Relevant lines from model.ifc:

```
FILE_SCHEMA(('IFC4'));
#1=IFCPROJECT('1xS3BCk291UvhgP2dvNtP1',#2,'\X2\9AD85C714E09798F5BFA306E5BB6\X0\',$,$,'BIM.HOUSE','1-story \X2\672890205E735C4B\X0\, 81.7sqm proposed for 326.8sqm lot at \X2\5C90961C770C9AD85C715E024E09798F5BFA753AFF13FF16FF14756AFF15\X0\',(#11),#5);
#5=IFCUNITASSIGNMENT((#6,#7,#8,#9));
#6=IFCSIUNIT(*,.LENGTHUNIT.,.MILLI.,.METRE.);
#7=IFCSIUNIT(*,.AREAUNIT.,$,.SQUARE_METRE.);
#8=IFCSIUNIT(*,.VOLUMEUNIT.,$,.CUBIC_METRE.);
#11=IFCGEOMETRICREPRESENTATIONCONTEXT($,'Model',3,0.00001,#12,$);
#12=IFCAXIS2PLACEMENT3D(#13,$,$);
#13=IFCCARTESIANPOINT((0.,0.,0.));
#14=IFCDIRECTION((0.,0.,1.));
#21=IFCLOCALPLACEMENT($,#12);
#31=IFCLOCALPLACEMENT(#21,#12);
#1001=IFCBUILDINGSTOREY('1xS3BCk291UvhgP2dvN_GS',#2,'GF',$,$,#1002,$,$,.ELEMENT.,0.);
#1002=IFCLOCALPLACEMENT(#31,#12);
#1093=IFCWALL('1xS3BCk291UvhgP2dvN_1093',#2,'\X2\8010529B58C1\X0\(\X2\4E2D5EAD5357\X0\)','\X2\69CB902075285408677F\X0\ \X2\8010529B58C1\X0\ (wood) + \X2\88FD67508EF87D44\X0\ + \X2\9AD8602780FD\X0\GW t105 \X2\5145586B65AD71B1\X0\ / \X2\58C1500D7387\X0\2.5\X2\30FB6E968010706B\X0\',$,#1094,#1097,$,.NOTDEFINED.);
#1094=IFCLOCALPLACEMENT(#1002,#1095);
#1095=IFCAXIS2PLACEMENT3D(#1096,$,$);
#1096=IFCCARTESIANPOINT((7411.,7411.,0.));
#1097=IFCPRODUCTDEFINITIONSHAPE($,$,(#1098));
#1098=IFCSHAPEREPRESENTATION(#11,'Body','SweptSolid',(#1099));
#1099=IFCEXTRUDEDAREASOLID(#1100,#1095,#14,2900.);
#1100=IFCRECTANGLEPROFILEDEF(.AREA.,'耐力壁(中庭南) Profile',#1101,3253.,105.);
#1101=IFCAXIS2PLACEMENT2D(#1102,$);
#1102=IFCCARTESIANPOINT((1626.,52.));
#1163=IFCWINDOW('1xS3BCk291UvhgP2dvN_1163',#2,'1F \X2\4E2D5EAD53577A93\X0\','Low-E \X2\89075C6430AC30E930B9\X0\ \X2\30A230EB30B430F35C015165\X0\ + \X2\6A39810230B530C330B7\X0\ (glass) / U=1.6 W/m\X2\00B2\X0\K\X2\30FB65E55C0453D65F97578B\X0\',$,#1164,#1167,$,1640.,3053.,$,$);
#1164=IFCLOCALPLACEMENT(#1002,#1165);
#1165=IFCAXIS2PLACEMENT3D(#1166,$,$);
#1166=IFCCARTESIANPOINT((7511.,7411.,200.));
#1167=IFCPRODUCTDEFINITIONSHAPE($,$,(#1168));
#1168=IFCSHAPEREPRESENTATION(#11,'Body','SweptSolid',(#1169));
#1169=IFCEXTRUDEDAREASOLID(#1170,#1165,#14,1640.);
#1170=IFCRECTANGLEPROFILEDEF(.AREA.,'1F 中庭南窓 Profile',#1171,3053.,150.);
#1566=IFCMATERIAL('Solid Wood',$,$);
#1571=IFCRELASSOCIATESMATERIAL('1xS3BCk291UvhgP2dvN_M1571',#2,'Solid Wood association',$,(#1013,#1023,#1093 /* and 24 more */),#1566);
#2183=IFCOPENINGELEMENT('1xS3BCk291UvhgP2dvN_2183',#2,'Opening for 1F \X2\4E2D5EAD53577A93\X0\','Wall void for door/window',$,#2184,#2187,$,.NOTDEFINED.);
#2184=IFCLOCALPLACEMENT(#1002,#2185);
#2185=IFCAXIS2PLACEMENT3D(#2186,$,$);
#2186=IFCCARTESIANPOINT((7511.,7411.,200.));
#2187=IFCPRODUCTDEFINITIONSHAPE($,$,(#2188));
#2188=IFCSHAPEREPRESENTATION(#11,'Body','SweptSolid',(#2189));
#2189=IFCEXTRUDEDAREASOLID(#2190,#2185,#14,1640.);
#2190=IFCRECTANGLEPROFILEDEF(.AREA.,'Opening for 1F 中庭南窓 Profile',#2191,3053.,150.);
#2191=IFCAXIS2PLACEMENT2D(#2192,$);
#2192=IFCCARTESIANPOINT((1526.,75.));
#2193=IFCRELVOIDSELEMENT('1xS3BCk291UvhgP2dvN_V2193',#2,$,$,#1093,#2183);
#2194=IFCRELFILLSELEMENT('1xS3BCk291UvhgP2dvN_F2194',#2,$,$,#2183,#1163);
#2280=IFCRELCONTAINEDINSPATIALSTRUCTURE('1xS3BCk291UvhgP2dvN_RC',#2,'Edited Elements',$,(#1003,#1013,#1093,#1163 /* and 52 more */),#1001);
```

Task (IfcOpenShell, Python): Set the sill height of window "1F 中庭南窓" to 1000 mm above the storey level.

```python
import numpy as np
import ifcopenshell
import ifcopenshell.api.geometry
import ifcopenshell.geom
import ifcopenshell.util.element
import ifcopenshell.util.placement
import ifcopenshell.util.shape
import ifcopenshell.util.unit

model = ifcopenshell.open("model.ifc")
unit_scale = ifcopenshell.util.unit.calculate_unit_scale(model)

window = model.by_guid("1xS3BCk291UvhgP2dvN_1163")
opening = window.FillsVoids[0].RelatingOpeningElement
storey = ifcopenshell.util.element.get_container(window, ifc_class="IfcBuildingStorey")
level = ifcopenshell.util.placement.get_local_placement(storey.ObjectPlacement)[2, 3]

# The opening's origin need not be at the sill, so measure its lowest point.
shape = ifcopenshell.geom.create_shape(ifcopenshell.geom.settings(), opening)
bottom = ifcopenshell.util.shape.get_shape_bottom_elevation(shape, shape.geometry) / unit_scale
dz = level + 1000.0 - bottom

shift = np.array([0.0, 0.0, dz])
# The window is not placed relative to its opening, so move both.
for product in (opening, window):
    matrix = ifcopenshell.util.placement.get_local_placement(product.ObjectPlacement)
    matrix[:3, 3] += shift
    ifcopenshell.api.geometry.edit_object_placement(model, product=product, matrix=matrix, is_si=False)

print(f"moved by {dz * unit_scale:+.3f} m")

model.write("model_updated.ifc")
```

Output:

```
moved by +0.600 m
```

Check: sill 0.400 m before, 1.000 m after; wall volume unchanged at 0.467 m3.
